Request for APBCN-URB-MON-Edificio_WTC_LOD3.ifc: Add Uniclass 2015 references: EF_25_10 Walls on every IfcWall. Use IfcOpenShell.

First a look at what the model holds.

```python
import ifcopenshell

model = ifcopenshell.open("APBCN-URB-MON-Edificio_WTC_LOD3.ifc")
print(model.schema)
print("classifications:", [c.Name for c in model.by_type("IfcClassification")])
for ifc_class in ("IfcDoor", "IfcRoof", "IfcStair", "IfcWall", "IfcWindow"):
    print(ifc_class, len(model.by_type(ifc_class)))
```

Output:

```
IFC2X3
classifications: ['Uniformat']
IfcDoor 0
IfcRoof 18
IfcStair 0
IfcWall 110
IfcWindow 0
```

```python
import ifcopenshell
import ifcopenshell.api.classification

model = ifcopenshell.open("APBCN-URB-MON-Edificio_WTC_LOD3.ifc")

# IFC2X3 requires Source and Edition and has no link from the project to the system.
system = model.create_entity("IfcClassification", Source="NBS", Edition="2015", Name="Uniclass 2015")

codes = {
    "IfcWall": ("EF_25_10", "Walls"),
}
for ifc_class, (code, name) in codes.items():
    products = model.by_type(ifc_class)
    ifcopenshell.api.classification.add_reference(
        model, products=products, classification=system, identification=code, name=name
    )
    print(code, len(products))

model.write("APBCN-URB-MON-Edificio_WTC_LOD3_v2.ifc")
```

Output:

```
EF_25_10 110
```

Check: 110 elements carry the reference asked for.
